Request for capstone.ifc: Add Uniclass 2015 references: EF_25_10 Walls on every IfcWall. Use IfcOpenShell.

First a look at what the model holds.

```python
import ifcopenshell

model = ifcopenshell.open("capstone.ifc")
print(model.schema)
print("classifications:", [c.Name for c in model.by_type("IfcClassification")])
for ifc_class in ("IfcDoor", "IfcRoof", "IfcStair", "IfcWall", "IfcWindow"):
    print(ifc_class, len(model.by_type(ifc_class)))
```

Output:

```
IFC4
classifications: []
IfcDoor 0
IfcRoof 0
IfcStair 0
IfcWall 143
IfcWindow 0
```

```python
import ifcopenshell
import ifcopenshell.api.classification

model = ifcopenshell.open("capstone.ifc")

system = ifcopenshell.api.classification.add_classification(model, classification="Uniclass 2015")

codes = {
    "IfcWall": ("EF_25_10", "Walls"),
}
for ifc_class, (code, name) in codes.items():
    products = model.by_type(ifc_class)
    ifcopenshell.api.classification.add_reference(
        model, products=products, classification=system, identification=code, name=name
    )
    print(code, len(products))

model.write("capstone_v2.ifc")
```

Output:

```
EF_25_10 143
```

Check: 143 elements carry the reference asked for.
